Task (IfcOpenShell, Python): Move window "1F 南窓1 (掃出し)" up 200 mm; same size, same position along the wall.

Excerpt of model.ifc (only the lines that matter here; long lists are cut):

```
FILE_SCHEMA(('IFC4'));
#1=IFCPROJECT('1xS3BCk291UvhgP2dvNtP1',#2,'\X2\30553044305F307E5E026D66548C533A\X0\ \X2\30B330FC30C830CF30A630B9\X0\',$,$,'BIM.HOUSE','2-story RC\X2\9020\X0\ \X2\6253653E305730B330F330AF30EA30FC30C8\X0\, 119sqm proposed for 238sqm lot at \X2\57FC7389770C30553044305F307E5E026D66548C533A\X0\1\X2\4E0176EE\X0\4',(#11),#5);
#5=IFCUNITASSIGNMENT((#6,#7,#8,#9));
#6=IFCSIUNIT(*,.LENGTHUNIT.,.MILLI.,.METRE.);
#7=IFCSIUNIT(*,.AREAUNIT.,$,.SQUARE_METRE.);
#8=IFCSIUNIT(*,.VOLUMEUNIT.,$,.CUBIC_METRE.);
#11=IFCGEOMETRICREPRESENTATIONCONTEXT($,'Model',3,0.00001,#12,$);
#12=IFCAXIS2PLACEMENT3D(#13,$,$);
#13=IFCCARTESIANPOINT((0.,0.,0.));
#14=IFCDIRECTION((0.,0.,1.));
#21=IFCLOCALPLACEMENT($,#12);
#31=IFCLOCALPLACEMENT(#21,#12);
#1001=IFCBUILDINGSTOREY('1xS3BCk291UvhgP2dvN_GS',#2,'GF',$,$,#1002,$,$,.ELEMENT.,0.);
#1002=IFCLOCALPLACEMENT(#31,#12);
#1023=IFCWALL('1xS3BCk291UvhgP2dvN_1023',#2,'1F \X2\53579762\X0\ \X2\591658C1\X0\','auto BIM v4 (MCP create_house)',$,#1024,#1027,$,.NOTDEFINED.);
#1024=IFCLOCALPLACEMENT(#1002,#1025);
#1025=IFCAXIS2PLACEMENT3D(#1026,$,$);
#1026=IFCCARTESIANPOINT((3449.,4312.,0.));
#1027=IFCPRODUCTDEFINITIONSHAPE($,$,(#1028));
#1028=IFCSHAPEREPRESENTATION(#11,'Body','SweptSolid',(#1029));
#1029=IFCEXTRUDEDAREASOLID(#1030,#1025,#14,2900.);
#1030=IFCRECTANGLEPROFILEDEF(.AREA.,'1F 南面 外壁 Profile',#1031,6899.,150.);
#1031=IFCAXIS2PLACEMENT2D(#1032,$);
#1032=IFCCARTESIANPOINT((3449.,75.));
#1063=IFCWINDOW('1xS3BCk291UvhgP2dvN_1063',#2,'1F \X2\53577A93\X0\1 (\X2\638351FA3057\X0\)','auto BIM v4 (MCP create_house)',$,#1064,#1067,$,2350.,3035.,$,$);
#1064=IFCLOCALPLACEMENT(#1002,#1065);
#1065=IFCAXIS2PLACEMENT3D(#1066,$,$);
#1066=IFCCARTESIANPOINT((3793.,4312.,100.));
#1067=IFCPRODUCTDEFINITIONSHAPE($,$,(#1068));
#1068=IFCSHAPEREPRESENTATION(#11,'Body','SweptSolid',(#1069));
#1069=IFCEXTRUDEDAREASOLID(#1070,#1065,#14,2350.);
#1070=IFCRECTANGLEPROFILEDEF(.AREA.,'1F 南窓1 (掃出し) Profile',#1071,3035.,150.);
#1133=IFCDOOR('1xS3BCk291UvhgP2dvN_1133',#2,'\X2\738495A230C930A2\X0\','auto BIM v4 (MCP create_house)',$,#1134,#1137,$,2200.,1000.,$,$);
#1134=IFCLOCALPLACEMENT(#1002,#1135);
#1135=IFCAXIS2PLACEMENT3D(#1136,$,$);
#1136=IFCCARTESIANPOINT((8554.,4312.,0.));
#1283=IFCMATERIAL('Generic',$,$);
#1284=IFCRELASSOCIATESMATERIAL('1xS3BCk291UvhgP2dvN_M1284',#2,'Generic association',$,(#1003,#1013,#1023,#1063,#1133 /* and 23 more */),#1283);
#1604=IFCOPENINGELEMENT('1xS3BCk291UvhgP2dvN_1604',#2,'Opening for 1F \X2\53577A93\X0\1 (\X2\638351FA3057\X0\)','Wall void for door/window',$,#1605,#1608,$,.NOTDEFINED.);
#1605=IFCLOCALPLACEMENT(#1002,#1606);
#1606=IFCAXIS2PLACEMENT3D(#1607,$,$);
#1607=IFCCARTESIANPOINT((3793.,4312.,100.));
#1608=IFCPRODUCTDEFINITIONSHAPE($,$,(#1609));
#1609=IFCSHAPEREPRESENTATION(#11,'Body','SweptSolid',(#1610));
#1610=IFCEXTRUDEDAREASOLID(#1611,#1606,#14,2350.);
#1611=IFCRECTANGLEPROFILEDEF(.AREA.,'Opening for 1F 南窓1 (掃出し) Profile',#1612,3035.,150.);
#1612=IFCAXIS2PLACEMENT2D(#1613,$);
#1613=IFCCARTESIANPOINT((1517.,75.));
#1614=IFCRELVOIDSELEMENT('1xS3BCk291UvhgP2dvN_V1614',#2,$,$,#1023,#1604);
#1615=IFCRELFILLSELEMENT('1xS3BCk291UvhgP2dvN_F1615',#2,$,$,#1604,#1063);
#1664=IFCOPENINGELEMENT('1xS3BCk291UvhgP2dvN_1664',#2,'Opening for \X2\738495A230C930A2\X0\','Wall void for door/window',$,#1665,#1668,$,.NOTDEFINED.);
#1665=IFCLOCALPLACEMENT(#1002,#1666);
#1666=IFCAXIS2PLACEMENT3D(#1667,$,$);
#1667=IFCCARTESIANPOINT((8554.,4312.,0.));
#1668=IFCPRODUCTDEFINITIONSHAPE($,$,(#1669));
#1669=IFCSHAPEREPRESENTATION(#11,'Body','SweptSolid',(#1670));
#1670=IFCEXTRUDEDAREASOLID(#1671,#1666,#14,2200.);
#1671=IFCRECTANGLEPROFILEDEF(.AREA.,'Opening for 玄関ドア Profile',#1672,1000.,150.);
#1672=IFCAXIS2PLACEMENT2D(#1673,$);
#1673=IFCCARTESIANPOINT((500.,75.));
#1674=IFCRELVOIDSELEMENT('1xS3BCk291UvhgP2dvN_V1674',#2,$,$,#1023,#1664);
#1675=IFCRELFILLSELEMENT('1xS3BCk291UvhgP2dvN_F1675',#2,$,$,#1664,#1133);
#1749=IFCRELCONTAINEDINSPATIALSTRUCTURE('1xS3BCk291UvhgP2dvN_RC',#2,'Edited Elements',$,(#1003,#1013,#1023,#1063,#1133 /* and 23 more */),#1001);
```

```python
import numpy as np
import ifcopenshell
import ifcopenshell.api.geometry
import ifcopenshell.util.placement
import ifcopenshell.util.unit

model = ifcopenshell.open("model.ifc")
unit_scale = ifcopenshell.util.unit.calculate_unit_scale(model)

window = model.by_guid("1xS3BCk291UvhgP2dvN_1063")
opening = window.FillsVoids[0].RelatingOpeningElement
dz = 0.2 / unit_scale

shift = np.array([0.0, 0.0, dz])
# The window is not placed relative to its opening, so move both.
for product in (opening, window):
    matrix = ifcopenshell.util.placement.get_local_placement(product.ObjectPlacement)
    matrix[:3, 3] += shift
    ifcopenshell.api.geometry.edit_object_placement(model, product=product, matrix=matrix, is_si=False)

print(f"moved by {dz * unit_scale:+.3f} m")

model.write("model_v2.ifc")
```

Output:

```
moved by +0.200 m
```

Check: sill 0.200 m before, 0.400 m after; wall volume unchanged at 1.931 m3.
